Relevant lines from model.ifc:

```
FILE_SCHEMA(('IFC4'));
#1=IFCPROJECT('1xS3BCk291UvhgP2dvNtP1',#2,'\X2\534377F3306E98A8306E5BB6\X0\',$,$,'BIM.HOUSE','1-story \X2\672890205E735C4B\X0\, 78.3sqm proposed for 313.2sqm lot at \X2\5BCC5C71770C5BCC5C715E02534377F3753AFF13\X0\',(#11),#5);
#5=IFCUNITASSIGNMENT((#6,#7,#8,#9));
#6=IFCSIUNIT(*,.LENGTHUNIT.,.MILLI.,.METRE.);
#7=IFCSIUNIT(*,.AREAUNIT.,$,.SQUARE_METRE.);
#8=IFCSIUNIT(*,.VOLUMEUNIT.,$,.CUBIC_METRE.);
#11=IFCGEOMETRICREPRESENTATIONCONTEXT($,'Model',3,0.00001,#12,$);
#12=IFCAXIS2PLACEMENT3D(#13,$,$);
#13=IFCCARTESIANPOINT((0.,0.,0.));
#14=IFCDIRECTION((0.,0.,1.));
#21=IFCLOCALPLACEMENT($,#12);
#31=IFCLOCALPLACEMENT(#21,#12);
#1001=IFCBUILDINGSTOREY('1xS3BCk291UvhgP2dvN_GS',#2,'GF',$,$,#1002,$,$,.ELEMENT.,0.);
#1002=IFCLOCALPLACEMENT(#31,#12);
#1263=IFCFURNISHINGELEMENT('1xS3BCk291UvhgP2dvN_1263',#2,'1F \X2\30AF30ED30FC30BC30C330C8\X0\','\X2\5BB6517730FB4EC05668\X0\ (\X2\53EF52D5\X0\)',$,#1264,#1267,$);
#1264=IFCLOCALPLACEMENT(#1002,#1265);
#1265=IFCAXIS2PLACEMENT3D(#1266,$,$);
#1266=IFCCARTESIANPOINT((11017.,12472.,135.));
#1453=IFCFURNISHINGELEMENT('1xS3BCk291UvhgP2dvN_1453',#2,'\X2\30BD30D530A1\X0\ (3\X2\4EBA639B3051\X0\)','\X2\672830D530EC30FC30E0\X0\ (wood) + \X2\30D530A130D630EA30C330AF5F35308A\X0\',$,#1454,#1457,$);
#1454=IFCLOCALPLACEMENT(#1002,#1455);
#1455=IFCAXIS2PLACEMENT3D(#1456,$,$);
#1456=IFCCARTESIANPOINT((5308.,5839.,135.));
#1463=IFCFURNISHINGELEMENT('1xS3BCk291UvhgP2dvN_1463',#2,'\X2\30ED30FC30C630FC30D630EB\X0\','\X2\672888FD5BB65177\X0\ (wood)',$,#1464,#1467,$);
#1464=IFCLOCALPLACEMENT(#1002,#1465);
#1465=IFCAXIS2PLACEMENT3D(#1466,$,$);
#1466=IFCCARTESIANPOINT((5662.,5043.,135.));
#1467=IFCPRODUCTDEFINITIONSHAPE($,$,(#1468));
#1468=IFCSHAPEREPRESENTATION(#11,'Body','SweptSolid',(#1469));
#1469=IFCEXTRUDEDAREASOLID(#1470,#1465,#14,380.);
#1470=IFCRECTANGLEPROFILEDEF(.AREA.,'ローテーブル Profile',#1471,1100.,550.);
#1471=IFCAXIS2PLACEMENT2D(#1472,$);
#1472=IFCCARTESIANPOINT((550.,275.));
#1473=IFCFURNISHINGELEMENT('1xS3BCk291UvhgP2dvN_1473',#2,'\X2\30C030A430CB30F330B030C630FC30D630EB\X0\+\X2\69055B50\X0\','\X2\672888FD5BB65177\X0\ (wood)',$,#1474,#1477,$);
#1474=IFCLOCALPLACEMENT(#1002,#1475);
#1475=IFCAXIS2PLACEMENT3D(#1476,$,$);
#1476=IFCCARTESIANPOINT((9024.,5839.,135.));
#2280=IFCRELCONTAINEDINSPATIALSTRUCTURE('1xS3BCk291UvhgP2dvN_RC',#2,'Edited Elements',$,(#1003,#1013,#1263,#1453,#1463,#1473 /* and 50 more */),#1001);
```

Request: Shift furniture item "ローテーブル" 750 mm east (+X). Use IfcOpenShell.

```python
import ifcopenshell
import ifcopenshell.api.geometry
import ifcopenshell.util.placement

model = ifcopenshell.open("model.ifc")

item = model.by_id(1463)
matrix = ifcopenshell.util.placement.get_local_placement(item.ObjectPlacement)
matrix[0, 3] += 750.0
ifcopenshell.api.geometry.edit_object_placement(model, product=item, matrix=matrix, is_si=False)

print(ifcopenshell.util.placement.get_local_placement(item.ObjectPlacement).round(3) + 0.0)

model.write("model_rev.ifc")
```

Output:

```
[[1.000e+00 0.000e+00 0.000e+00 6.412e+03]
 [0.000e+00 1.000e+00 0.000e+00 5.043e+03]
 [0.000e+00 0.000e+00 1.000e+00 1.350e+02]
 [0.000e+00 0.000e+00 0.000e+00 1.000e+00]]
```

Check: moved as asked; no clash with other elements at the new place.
